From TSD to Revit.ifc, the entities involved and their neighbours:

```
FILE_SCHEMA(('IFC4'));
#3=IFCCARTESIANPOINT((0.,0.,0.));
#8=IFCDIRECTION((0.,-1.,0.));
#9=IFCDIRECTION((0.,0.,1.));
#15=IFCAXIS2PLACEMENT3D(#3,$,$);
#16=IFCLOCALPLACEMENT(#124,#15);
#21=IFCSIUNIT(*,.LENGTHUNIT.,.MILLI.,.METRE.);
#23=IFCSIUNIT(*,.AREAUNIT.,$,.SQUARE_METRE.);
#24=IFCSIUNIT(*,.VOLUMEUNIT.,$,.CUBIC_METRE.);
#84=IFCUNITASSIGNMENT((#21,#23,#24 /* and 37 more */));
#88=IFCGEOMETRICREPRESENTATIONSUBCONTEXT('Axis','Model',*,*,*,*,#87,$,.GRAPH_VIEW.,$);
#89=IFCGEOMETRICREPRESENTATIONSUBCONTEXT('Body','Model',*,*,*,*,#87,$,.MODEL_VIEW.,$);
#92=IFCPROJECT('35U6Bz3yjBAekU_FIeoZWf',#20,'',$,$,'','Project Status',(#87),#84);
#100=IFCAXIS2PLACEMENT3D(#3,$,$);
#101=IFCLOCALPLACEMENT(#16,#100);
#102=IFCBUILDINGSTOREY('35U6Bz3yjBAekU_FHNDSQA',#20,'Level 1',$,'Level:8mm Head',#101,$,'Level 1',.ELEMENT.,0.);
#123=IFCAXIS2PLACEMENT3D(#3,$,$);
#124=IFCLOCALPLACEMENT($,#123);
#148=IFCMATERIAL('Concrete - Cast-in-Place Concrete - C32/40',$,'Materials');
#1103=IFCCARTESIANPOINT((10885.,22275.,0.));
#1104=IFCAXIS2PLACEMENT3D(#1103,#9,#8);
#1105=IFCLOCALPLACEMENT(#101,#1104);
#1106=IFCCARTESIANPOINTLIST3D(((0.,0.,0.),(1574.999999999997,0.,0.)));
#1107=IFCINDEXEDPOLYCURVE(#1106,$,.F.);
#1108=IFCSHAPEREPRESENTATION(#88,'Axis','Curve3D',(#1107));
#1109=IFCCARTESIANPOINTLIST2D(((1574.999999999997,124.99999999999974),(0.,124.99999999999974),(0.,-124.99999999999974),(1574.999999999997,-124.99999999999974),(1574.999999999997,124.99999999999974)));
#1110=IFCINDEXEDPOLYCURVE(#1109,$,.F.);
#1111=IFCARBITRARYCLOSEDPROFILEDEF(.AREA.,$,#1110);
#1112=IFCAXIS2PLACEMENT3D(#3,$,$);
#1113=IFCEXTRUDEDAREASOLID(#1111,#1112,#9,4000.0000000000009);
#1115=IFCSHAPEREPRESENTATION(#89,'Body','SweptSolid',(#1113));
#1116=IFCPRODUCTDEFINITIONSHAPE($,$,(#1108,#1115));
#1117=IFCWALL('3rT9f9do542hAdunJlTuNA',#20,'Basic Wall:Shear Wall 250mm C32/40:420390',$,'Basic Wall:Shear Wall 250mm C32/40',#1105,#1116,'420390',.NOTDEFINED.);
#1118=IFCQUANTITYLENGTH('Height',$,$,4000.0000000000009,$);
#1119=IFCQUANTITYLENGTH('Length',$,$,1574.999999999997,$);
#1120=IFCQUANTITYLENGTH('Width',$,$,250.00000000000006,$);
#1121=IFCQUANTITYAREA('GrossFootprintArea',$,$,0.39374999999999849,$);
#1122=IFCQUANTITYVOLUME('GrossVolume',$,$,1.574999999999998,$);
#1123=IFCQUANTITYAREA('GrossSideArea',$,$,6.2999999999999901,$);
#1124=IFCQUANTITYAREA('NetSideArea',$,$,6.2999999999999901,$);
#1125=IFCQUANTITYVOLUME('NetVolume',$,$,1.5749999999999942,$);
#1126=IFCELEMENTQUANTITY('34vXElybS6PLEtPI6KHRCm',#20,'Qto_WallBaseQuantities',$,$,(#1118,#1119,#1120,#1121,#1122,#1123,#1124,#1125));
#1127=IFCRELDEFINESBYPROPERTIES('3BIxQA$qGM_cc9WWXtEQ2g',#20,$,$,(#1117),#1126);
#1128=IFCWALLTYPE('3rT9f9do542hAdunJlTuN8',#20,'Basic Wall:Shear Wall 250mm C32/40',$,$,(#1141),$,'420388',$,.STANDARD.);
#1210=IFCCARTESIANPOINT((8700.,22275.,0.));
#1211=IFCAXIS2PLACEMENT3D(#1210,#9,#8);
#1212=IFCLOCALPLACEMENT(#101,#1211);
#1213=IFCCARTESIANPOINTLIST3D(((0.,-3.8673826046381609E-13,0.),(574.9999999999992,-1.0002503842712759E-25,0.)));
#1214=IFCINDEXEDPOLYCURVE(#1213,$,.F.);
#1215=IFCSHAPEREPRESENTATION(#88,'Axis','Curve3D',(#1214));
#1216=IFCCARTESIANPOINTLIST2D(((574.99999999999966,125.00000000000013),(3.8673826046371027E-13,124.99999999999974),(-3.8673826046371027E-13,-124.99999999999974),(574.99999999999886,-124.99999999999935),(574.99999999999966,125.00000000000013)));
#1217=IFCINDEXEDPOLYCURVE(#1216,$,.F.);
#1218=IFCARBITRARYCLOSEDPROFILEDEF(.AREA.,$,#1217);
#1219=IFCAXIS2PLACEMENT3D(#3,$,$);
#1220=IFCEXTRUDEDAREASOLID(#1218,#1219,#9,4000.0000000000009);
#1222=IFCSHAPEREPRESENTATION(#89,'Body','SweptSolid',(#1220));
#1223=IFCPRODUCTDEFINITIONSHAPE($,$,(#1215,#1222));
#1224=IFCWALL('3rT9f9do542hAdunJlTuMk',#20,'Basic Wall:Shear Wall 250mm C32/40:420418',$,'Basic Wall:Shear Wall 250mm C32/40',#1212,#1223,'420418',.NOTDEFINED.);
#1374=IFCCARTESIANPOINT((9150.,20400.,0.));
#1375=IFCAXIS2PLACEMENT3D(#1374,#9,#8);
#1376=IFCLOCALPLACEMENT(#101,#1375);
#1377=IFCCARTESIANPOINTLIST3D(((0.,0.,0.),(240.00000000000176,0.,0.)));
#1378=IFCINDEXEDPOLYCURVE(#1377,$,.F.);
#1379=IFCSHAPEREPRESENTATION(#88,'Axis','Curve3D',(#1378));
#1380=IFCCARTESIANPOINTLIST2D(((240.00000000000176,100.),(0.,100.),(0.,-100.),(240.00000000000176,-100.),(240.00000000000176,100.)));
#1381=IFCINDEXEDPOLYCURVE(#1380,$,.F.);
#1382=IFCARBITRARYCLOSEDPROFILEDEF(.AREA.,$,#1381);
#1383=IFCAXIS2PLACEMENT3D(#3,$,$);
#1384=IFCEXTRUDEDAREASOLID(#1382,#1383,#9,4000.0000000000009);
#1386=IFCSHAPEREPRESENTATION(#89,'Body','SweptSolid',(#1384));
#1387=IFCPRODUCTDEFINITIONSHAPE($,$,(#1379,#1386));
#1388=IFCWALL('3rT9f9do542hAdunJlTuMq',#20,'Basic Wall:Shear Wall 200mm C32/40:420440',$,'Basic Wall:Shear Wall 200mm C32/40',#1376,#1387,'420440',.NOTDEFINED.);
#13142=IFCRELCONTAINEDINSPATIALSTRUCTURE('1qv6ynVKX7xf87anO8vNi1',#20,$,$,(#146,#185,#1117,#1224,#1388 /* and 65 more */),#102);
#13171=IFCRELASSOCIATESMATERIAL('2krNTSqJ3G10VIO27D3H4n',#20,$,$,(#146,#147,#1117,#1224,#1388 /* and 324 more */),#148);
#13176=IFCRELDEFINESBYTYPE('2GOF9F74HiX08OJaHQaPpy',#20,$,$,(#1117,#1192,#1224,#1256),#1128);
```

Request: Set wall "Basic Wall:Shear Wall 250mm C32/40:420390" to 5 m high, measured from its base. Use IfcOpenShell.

```python
import ifcopenshell
import ifcopenshell.api.pset
import ifcopenshell.geom
import ifcopenshell.util.element
import ifcopenshell.util.representation
import ifcopenshell.util.shape
import ifcopenshell.util.unit

model = ifcopenshell.open("TSD to Revit.ifc")
unit_scale = ifcopenshell.util.unit.calculate_unit_scale(model)
area_scale = ifcopenshell.util.unit.calculate_unit_scale(model, "AREAUNIT")
volume_scale = ifcopenshell.util.unit.calculate_unit_scale(model, "VOLUMEUNIT")
settings = ifcopenshell.geom.settings()


def volume(element):
    """Net volume in cubic metres, openings subtracted."""
    shape = ifcopenshell.geom.create_shape(settings, element)
    return ifcopenshell.util.shape.get_volume(shape.geometry)


wall = model.by_guid("3rT9f9do542hAdunJlTuNA")
before = volume(wall)

body = ifcopenshell.util.representation.get_representation(wall, "Model", "Body")
solid = body.Items[0]
old_height = solid.Depth
solid.Depth = 5000.0
after = volume(wall)
thickness = 0.25  # wall thickness in metres

# Update the stored height, areas and volumes.
qto = model.by_id(ifcopenshell.util.element.get_pset(wall, "Qto_WallBaseQuantities", should_inherit=False)["id"])
ifcopenshell.api.pset.edit_qto(model, qto=qto, properties={
    "Height": solid.Depth,
    "GrossVolume": ifcopenshell.util.element.get_pset(wall, "Qto_WallBaseQuantities", "GrossVolume") * solid.Depth / old_height,
    "GrossSideArea": ifcopenshell.util.element.get_pset(wall, "Qto_WallBaseQuantities", "GrossSideArea") * solid.Depth / old_height,
    "NetSideArea": after / thickness / area_scale,
    "NetVolume": after / volume_scale,
})

print(f"height {old_height:g} -> {solid.Depth:g}, volume {before:.3f} -> {after:.3f} m3")

model.write("TSD to Revit_updated.ifc")
```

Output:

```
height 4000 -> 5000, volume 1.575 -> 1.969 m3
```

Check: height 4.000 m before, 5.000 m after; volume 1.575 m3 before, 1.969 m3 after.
